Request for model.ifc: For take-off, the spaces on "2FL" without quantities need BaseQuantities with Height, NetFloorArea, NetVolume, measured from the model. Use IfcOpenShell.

First a look at what the model holds.

```python
import ifcopenshell
import ifcopenshell.util.element
import ifcopenshell.util.unit

model = ifcopenshell.open("model.ifc")
print(model.schema)
for unit_type in ("LENGTHUNIT", "AREAUNIT", "VOLUMEUNIT"):
    print(unit_type, ifcopenshell.util.unit.calculate_unit_scale(model, unit_type))
storey = next(s for s in model.by_type("IfcBuildingStorey") if s.Name == "2FL")
spaces = [e for e in ifcopenshell.util.element.get_decomposition(storey) if e.is_a("IfcSpace")]
for e in sorted(spaces, key=lambda e: e.id()):
    print(e.id(), e.is_a(), e.Name, list(ifcopenshell.util.element.get_psets(e, qtos_only=True)), sep=" | ")
```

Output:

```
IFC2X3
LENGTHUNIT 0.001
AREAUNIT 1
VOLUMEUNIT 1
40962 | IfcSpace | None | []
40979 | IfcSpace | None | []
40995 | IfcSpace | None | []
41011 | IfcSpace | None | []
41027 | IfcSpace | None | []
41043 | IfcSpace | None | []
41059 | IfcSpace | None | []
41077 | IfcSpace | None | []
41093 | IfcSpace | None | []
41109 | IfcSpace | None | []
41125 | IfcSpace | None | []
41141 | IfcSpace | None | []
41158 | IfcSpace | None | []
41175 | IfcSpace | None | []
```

```python
import ifcopenshell
import ifcopenshell.api.pset
import ifcopenshell.geom
import ifcopenshell.util.element
import ifcopenshell.util.shape
import ifcopenshell.util.unit

model = ifcopenshell.open("model.ifc")
unit_scale = ifcopenshell.util.unit.calculate_unit_scale(model)
area_scale = ifcopenshell.util.unit.calculate_unit_scale(model, "AREAUNIT")
volume_scale = ifcopenshell.util.unit.calculate_unit_scale(model, "VOLUMEUNIT")
settings = ifcopenshell.geom.settings()

storey = next(s for s in model.by_type("IfcBuildingStorey") if s.Name == "2FL")
spaces = [e for e in ifcopenshell.util.element.get_decomposition(storey) if e.is_a("IfcSpace")]

for e in sorted(spaces, key=lambda e: e.id()):
    if ifcopenshell.util.element.get_psets(e, qtos_only=True, should_inherit=False):
        continue
    # Geometry comes back in metres, in the element's own axes.
    shape = ifcopenshell.geom.create_shape(settings, e)
    values = {
        "Height": ifcopenshell.util.shape.get_z(shape.geometry) / unit_scale,
        "NetFloorArea": ifcopenshell.util.shape.get_footprint_area(shape.geometry) / area_scale,
        "NetVolume": ifcopenshell.util.shape.get_volume(shape.geometry) / volume_scale,
    }
    qto = ifcopenshell.api.pset.add_qto(model, product=e, name="BaseQuantities")
    ifcopenshell.api.pset.edit_qto(model, qto=qto, properties=values)
    print(e.id(), {k: round(v, 3) for k, v in values.items()})

model.write("model-out.ifc")
```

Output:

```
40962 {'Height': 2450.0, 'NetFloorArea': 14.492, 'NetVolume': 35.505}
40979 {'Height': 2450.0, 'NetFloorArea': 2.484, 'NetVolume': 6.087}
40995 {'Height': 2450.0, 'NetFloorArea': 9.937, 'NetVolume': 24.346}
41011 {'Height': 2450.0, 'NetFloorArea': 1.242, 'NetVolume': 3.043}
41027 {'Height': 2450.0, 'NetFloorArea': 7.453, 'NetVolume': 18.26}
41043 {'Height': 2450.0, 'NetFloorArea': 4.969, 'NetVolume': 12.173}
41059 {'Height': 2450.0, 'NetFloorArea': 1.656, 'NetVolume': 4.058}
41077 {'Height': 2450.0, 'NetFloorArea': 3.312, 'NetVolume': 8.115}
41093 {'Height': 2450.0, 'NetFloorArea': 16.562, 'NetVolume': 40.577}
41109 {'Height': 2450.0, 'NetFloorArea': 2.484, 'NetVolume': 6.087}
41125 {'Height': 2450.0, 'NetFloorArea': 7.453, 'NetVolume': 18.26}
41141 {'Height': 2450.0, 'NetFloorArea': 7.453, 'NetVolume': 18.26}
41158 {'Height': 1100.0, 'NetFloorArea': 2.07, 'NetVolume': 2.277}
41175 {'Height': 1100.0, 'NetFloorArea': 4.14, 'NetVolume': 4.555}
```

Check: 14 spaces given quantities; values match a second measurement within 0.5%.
